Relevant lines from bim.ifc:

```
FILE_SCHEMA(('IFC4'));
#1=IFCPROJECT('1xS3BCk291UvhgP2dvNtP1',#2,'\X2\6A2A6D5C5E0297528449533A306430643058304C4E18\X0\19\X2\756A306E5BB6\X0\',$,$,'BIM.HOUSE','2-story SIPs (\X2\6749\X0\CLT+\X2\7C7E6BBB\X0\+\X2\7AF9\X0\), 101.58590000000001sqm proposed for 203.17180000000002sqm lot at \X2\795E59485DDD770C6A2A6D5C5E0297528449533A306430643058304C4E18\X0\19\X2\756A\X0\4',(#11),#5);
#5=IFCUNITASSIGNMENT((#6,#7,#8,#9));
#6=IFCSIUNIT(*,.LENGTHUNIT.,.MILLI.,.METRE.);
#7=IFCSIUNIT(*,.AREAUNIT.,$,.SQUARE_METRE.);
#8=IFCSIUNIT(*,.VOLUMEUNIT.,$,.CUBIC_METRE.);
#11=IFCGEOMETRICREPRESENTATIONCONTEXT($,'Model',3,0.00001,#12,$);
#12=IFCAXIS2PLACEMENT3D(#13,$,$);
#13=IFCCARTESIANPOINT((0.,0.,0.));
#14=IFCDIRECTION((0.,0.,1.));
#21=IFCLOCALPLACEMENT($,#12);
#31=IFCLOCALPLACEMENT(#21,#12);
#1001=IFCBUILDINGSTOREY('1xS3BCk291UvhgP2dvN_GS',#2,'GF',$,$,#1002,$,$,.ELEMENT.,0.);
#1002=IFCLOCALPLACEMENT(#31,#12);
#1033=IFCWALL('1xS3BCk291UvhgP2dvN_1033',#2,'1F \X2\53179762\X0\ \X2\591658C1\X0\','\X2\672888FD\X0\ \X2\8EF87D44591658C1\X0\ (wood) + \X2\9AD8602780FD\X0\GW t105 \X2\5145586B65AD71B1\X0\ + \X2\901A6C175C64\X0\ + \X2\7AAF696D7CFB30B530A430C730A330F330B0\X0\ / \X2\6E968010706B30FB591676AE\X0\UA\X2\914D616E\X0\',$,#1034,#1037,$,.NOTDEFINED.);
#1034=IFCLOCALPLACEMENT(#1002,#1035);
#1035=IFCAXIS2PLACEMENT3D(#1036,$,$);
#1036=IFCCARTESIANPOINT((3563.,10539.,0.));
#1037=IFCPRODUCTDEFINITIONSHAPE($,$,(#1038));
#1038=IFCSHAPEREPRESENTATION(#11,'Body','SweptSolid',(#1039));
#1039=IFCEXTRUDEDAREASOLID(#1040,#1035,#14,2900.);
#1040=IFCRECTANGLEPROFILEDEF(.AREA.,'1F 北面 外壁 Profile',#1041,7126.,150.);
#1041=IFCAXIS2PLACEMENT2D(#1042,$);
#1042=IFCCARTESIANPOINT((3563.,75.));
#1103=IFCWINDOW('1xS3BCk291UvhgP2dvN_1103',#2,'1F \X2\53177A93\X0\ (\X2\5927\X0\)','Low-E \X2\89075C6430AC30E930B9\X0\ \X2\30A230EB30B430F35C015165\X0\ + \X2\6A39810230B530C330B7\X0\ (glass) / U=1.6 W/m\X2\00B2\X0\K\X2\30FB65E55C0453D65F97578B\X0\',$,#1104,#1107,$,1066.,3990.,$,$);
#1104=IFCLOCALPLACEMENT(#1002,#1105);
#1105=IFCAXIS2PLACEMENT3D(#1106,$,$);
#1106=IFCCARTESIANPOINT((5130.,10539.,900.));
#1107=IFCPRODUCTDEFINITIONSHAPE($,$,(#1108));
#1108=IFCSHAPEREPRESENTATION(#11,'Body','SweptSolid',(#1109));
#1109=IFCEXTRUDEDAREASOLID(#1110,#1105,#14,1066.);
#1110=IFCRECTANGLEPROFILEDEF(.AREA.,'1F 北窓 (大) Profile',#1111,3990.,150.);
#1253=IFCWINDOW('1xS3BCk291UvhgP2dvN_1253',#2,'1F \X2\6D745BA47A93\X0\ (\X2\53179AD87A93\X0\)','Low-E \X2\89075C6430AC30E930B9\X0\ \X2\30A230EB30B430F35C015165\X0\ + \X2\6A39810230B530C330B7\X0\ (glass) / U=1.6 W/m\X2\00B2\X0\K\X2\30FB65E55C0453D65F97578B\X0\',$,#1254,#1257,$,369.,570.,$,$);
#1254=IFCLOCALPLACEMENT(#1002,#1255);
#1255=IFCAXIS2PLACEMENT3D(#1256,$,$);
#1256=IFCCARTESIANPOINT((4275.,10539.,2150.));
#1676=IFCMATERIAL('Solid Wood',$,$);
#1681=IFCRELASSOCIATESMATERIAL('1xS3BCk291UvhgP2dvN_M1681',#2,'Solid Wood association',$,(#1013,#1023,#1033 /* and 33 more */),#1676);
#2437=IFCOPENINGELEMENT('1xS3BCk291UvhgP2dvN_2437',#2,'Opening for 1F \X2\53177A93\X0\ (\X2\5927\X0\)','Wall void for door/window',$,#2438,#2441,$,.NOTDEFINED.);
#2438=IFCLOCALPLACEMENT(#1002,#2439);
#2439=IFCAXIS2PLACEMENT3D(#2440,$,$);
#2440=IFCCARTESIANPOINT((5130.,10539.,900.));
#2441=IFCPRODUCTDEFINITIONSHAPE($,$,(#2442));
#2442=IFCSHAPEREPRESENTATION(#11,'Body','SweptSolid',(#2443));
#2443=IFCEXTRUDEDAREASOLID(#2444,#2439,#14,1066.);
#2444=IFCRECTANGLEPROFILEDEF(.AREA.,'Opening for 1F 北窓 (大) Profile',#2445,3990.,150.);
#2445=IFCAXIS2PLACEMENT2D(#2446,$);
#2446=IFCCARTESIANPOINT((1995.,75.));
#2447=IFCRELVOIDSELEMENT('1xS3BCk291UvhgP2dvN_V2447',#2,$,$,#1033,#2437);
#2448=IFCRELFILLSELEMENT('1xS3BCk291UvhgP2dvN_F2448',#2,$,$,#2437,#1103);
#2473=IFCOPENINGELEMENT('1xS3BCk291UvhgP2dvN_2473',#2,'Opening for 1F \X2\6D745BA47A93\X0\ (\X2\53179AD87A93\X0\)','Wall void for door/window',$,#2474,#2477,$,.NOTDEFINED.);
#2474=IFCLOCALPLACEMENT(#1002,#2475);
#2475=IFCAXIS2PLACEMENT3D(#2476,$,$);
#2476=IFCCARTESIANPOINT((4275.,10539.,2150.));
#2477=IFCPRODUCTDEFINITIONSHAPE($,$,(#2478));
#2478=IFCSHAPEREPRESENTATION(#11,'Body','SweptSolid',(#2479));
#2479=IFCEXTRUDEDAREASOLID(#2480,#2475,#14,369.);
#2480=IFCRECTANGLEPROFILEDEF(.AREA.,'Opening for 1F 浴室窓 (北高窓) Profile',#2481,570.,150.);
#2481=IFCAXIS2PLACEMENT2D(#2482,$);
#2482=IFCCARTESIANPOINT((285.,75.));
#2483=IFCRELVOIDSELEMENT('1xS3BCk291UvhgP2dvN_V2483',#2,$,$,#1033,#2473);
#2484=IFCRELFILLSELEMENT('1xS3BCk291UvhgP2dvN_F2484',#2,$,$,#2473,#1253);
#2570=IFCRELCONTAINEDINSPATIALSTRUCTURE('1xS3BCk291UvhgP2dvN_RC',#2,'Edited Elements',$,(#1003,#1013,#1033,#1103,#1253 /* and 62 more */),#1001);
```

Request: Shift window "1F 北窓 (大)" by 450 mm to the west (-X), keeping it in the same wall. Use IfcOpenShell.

```python
import ifcopenshell
import ifcopenshell.api.geometry
import ifcopenshell.util.placement
import ifcopenshell.util.unit

model = ifcopenshell.open("bim.ifc")
unit_scale = ifcopenshell.util.unit.calculate_unit_scale(model)

window = model.by_guid("1xS3BCk291UvhgP2dvN_1103")
opening = window.FillsVoids[0].RelatingOpeningElement
wall = opening.VoidsElements[0].RelatingBuildingElement

wall_matrix = ifcopenshell.util.placement.get_local_placement(wall.ObjectPlacement)
shift = wall_matrix[:3, 0] * -0.45 / unit_scale
before = ifcopenshell.util.placement.get_local_placement(window.ObjectPlacement)[:3, 3].copy()

# The window is not placed relative to its opening, so move both.
for product in (opening, window):
    matrix = ifcopenshell.util.placement.get_local_placement(product.ObjectPlacement)
    matrix[:3, 3] += shift
    ifcopenshell.api.geometry.edit_object_placement(model, product=product, matrix=matrix, is_si=False)

after = ifcopenshell.util.placement.get_local_placement(window.ObjectPlacement)[:3, 3]
print("window moved by", (after - before).round(3) + 0.0)

model.write("bim_updated.ifc")
```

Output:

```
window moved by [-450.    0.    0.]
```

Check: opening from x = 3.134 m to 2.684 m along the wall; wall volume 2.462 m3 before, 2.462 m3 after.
